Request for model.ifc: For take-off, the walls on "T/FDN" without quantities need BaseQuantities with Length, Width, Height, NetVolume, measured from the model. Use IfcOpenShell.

First a look at what the model holds.

```python
import ifcopenshell
import ifcopenshell.util.element
import ifcopenshell.util.unit

model = ifcopenshell.open("model.ifc")
print(model.schema)
for unit_type in ("LENGTHUNIT", "AREAUNIT", "VOLUMEUNIT"):
    print(unit_type, ifcopenshell.util.unit.calculate_unit_scale(model, unit_type))
storey = next(s for s in model.by_type("IfcBuildingStorey") if s.Name == "T/FDN")
walls = [e for e in ifcopenshell.util.element.get_decomposition(storey) if e.is_a("IfcWall")]
for e in sorted(walls, key=lambda e: e.id()):
    print(e.id(), e.is_a(), e.Name, list(ifcopenshell.util.element.get_psets(e, qtos_only=True)), sep=" | ")
```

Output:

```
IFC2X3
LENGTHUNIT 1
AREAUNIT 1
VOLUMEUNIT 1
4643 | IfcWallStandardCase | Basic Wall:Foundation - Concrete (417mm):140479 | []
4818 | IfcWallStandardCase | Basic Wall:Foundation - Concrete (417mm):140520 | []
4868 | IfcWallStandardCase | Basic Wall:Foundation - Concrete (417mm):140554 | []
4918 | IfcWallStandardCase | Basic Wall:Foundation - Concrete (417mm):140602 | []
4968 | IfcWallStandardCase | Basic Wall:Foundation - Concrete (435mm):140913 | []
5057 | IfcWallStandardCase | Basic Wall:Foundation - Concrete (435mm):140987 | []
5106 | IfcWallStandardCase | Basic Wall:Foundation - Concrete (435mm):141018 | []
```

```python
import ifcopenshell
import ifcopenshell.api.pset
import ifcopenshell.geom
import ifcopenshell.util.element
import ifcopenshell.util.shape
import ifcopenshell.util.unit

model = ifcopenshell.open("model.ifc")
unit_scale = ifcopenshell.util.unit.calculate_unit_scale(model)
volume_scale = ifcopenshell.util.unit.calculate_unit_scale(model, "VOLUMEUNIT")
settings = ifcopenshell.geom.settings()

storey = next(s for s in model.by_type("IfcBuildingStorey") if s.Name == "T/FDN")
walls = [e for e in ifcopenshell.util.element.get_decomposition(storey) if e.is_a("IfcWall")]

for e in sorted(walls, key=lambda e: e.id()):
    if ifcopenshell.util.element.get_psets(e, qtos_only=True, should_inherit=False):
        continue
    # Geometry comes back in metres, in the element's own axes.
    shape = ifcopenshell.geom.create_shape(settings, e)
    values = {
        "Length": ifcopenshell.util.shape.get_x(shape.geometry) / unit_scale,
        "Width": ifcopenshell.util.shape.get_y(shape.geometry) / unit_scale,
        "Height": ifcopenshell.util.shape.get_z(shape.geometry) / unit_scale,
        "NetVolume": ifcopenshell.util.shape.get_volume(shape.geometry) / volume_scale,
    }
    qto = ifcopenshell.api.pset.add_qto(model, product=e, name="BaseQuantities")
    ifcopenshell.api.pset.edit_qto(model, qto=qto, properties=values)
    print(e.id(), {k: round(v, 3) for k, v in values.items()})

model.write("model_edited.ifc")
```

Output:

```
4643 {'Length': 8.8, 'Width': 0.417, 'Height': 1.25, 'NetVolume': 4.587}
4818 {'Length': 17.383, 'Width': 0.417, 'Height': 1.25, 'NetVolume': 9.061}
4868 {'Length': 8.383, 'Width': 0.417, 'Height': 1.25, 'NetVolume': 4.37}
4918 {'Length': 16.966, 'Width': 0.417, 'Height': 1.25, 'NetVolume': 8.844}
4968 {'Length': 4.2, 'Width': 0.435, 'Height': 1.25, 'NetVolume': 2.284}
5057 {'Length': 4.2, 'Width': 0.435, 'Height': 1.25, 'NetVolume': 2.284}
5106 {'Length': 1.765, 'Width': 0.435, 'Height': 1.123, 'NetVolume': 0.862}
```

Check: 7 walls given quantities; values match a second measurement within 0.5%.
